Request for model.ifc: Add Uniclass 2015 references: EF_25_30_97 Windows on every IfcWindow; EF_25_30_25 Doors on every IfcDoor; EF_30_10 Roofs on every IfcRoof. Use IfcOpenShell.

First a look at what the model holds.

```python
import ifcopenshell

model = ifcopenshell.open("model.ifc")
print(model.schema)
print("classifications:", [c.Name for c in model.by_type("IfcClassification")])
for ifc_class in ("IfcDoor", "IfcRoof", "IfcStair", "IfcWall", "IfcWindow"):
    print(ifc_class, len(model.by_type(ifc_class)))
```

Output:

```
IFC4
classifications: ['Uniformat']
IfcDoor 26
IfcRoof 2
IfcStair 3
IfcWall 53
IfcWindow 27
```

```python
import ifcopenshell
import ifcopenshell.api.classification

model = ifcopenshell.open("model.ifc")

system = ifcopenshell.api.classification.add_classification(model, classification="Uniclass 2015")

codes = {
    "IfcWindow": ("EF_25_30_97", "Windows"),
    "IfcDoor": ("EF_25_30_25", "Doors"),
    "IfcRoof": ("EF_30_10", "Roofs"),
}
for ifc_class, (code, name) in codes.items():
    products = model.by_type(ifc_class)
    ifcopenshell.api.classification.add_reference(
        model, products=products, classification=system, identification=code, name=name
    )
    print(code, len(products))

model.write("model_edited.ifc")
```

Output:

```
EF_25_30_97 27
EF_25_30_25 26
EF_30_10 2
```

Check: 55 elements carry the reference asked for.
